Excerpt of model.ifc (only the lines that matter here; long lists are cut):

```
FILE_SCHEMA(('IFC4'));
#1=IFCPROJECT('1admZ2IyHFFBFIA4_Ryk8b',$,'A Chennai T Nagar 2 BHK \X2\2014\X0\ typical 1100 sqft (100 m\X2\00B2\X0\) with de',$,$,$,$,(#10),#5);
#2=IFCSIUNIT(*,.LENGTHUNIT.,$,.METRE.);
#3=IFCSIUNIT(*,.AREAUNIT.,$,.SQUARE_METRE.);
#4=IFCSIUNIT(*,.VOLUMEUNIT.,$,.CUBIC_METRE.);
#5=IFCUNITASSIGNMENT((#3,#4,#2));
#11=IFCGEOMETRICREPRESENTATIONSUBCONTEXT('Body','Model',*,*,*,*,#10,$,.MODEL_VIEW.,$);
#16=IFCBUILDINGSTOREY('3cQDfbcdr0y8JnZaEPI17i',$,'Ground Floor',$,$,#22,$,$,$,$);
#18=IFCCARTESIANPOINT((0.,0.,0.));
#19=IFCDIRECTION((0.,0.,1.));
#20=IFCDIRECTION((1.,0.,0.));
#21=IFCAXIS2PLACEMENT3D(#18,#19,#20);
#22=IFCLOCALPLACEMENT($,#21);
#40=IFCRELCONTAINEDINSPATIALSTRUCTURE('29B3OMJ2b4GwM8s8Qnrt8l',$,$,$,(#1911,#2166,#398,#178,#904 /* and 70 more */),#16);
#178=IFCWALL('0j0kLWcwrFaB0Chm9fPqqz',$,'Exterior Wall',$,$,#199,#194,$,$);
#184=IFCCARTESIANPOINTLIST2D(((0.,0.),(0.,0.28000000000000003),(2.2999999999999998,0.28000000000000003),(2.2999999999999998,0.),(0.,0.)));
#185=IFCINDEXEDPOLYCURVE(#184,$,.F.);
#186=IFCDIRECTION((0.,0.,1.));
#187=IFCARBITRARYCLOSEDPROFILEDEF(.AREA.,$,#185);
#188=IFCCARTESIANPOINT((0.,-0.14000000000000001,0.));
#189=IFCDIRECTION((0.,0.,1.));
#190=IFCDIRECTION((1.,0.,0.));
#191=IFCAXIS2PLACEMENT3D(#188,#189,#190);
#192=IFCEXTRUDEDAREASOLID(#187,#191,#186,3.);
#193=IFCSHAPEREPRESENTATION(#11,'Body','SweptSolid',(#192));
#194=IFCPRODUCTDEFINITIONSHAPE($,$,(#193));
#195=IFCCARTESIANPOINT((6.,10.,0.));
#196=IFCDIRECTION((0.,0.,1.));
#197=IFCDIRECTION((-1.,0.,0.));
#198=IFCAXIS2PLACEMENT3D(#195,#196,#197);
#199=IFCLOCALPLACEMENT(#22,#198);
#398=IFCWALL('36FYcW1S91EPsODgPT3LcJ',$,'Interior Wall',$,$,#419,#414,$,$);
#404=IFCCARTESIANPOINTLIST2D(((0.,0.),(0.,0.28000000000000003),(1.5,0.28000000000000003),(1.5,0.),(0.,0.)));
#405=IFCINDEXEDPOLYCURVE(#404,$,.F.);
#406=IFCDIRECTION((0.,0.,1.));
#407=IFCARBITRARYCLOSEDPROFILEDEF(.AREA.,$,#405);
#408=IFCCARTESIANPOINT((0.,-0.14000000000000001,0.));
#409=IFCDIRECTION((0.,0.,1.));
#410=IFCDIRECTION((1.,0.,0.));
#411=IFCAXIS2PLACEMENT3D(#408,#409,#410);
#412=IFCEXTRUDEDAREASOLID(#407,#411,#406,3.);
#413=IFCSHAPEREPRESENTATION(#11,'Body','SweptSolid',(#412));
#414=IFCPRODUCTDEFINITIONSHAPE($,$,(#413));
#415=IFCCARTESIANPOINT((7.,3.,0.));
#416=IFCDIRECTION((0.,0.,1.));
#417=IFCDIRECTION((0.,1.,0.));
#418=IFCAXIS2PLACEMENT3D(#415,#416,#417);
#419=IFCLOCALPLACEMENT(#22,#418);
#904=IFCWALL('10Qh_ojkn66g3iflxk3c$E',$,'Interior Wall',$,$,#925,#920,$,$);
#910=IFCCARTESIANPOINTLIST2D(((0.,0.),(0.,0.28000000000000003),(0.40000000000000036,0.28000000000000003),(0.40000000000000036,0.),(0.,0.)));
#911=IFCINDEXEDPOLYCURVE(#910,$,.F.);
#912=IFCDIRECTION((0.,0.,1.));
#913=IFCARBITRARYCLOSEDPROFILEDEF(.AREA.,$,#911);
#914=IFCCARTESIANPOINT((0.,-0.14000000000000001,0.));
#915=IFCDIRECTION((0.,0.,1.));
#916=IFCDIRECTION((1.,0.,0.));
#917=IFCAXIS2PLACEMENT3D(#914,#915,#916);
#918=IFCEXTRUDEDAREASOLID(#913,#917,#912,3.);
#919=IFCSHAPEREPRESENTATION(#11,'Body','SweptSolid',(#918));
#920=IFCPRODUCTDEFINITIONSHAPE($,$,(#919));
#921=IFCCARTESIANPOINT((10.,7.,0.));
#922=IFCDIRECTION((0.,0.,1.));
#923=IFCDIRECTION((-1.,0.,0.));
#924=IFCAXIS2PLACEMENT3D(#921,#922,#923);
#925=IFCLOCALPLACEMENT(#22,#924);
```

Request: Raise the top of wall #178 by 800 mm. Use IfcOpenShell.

```python
import ifcopenshell
import ifcopenshell.geom
import ifcopenshell.util.representation
import ifcopenshell.util.shape
import ifcopenshell.util.unit

model = ifcopenshell.open("model.ifc")
unit_scale = ifcopenshell.util.unit.calculate_unit_scale(model)
settings = ifcopenshell.geom.settings()


def volume(element):
    """Net volume in cubic metres, openings subtracted."""
    shape = ifcopenshell.geom.create_shape(settings, element)
    return ifcopenshell.util.shape.get_volume(shape.geometry)


wall = model.by_guid("0j0kLWcwrFaB0Chm9fPqqz")
before = volume(wall)

body = ifcopenshell.util.representation.get_representation(wall, "Model", "Body")
solid = body.Items[0]
old_height = solid.Depth
solid.Depth += 0.8 / unit_scale
after = volume(wall)

print(f"height {old_height:g} -> {solid.Depth:g}, volume {before:.3f} -> {after:.3f} m3")

model.write("model_rev.ifc")
```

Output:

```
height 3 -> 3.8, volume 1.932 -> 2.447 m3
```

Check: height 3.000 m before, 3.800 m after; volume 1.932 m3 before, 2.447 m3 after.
